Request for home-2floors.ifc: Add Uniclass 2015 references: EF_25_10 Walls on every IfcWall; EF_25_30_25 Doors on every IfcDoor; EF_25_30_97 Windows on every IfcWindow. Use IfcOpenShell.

First a look at what the model holds.

```python
import ifcopenshell

model = ifcopenshell.open("home-2floors.ifc")
print(model.schema)
print("classifications:", [c.Name for c in model.by_type("IfcClassification")])
for ifc_class in ("IfcDoor", "IfcRoof", "IfcStair", "IfcWall", "IfcWindow"):
    print(ifc_class, len(model.by_type(ifc_class)))
```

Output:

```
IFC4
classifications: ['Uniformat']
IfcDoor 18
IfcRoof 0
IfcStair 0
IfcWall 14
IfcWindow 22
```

```python
import ifcopenshell
import ifcopenshell.api.classification

model = ifcopenshell.open("home-2floors.ifc")

system = ifcopenshell.api.classification.add_classification(model, classification="Uniclass 2015")

codes = {
    "IfcWall": ("EF_25_10", "Walls"),
    "IfcDoor": ("EF_25_30_25", "Doors"),
    "IfcWindow": ("EF_25_30_97", "Windows"),
}
for ifc_class, (code, name) in codes.items():
    products = model.by_type(ifc_class)
    ifcopenshell.api.classification.add_reference(
        model, products=products, classification=system, identification=code, name=name
    )
    print(code, len(products))

model.write("home-2floors_updated.ifc")
```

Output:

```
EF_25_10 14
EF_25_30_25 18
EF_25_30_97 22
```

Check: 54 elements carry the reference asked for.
